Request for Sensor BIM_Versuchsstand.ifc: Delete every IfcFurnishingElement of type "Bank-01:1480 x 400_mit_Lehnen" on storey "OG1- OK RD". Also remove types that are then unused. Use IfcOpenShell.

First a look at what the model holds.

```python
import ifcopenshell
import ifcopenshell.util.element

model = ifcopenshell.open("Sensor BIM_Versuchsstand.ifc")
print(model.schema)
storey = next(s for s in model.by_type("IfcBuildingStorey") if s.Name == "OG1- OK RD")
furniture = [e for e in ifcopenshell.util.element.get_decomposition(storey) if e.is_a("IfcFurnishingElement")]
seen = {}
for e in furniture:
    element_type = ifcopenshell.util.element.get_type(e)
    name = element_type.Name if element_type not in (None, e) else None
    seen[name] = seen.get(name, 0) + 1
for name, count in sorted(seen.items(), key=str):
    print(count, "x", name)
```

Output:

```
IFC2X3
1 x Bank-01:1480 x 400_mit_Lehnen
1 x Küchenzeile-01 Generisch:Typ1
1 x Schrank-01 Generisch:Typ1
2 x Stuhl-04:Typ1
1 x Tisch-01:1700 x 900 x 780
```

```python
import ifcopenshell
import ifcopenshell.api.root
import ifcopenshell.util.element

model = ifcopenshell.open("Sensor BIM_Versuchsstand.ifc")

storey = next(s for s in model.by_type("IfcBuildingStorey") if s.Name == "OG1- OK RD")
furniture = [e for e in ifcopenshell.util.element.get_decomposition(storey) if e.is_a("IfcFurnishingElement")]
targets = [e for e in furniture if (t := ifcopenshell.util.element.get_type(e)) not in (None, e) and t.Name == "Bank-01:1480 x 400_mit_Lehnen"]
types = {ifcopenshell.util.element.get_type(e) for e in targets} - {None, *targets}

for e in targets:
    ifcopenshell.api.root.remove_product(model, product=e)
print(len(targets), "removed")

unused = [t for t in types if not ifcopenshell.util.element.get_types(t)]
for t in unused:
    ifcopenshell.api.root.remove_product(model, product=t)
print(len(unused), "unused types removed")

model.write("Sensor BIM_Versuchsstand_v2.ifc")
```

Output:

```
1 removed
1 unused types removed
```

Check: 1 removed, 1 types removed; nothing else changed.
